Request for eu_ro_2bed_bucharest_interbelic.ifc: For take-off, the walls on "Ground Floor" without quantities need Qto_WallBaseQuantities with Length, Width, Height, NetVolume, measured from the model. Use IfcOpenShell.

First a look at what the model holds.

```python
import ifcopenshell
import ifcopenshell.util.element
import ifcopenshell.util.unit

model = ifcopenshell.open("eu_ro_2bed_bucharest_interbelic.ifc")
print(model.schema)
for unit_type in ("LENGTHUNIT", "AREAUNIT", "VOLUMEUNIT"):
    print(unit_type, ifcopenshell.util.unit.calculate_unit_scale(model, unit_type))
storey = next(s for s in model.by_type("IfcBuildingStorey") if s.Name == "Ground Floor")
walls = [e for e in ifcopenshell.util.element.get_decomposition(storey) if e.is_a("IfcWall")]
for e in sorted(walls, key=lambda e: e.id()):
    print(e.id(), e.is_a(), e.Name, list(ifcopenshell.util.element.get_psets(e, qtos_only=True)), sep=" | ")
```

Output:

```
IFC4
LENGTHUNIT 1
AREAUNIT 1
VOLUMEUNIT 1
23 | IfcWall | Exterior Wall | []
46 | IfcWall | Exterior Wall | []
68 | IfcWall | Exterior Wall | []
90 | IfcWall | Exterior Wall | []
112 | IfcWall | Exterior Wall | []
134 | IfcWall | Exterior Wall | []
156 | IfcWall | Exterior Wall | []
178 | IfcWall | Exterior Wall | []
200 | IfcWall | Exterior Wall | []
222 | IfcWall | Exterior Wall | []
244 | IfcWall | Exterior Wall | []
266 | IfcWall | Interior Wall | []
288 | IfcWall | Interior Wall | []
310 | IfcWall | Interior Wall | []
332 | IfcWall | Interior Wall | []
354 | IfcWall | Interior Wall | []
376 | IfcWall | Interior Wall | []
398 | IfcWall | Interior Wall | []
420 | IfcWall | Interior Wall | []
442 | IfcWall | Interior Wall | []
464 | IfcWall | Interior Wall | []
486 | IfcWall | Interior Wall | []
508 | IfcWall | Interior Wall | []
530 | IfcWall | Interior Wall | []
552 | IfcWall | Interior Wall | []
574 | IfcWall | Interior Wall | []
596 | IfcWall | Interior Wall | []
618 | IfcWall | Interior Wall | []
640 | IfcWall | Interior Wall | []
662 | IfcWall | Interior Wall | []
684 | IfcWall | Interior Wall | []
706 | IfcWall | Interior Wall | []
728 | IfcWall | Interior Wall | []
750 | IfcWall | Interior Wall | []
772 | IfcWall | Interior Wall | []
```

```python
import ifcopenshell
import ifcopenshell.api.pset
import ifcopenshell.geom
import ifcopenshell.util.element
import ifcopenshell.util.shape
import ifcopenshell.util.unit

model = ifcopenshell.open("eu_ro_2bed_bucharest_interbelic.ifc")
unit_scale = ifcopenshell.util.unit.calculate_unit_scale(model)
volume_scale = ifcopenshell.util.unit.calculate_unit_scale(model, "VOLUMEUNIT")
settings = ifcopenshell.geom.settings()

storey = next(s for s in model.by_type("IfcBuildingStorey") if s.Name == "Ground Floor")
walls = [e for e in ifcopenshell.util.element.get_decomposition(storey) if e.is_a("IfcWall")]

for e in sorted(walls, key=lambda e: e.id()):
    if ifcopenshell.util.element.get_psets(e, qtos_only=True, should_inherit=False):
        continue
    # Geometry comes back in metres, in the element's own axes.
    shape = ifcopenshell.geom.create_shape(settings, e)
    values = {
        "Length": ifcopenshell.util.shape.get_x(shape.geometry) / unit_scale,
        "Width": ifcopenshell.util.shape.get_y(shape.geometry) / unit_scale,
        "Height": ifcopenshell.util.shape.get_z(shape.geometry) / unit_scale,
        "NetVolume": ifcopenshell.util.shape.get_volume(shape.geometry) / volume_scale,
    }
    qto = ifcopenshell.api.pset.add_qto(model, product=e, name="Qto_WallBaseQuantities")
    ifcopenshell.api.pset.edit_qto(model, qto=qto, properties=values)
    print(e.id(), {k: round(v, 3) for k, v in values.items()})

model.write("eu_ro_2bed_bucharest_interbelic_updated.ifc")
```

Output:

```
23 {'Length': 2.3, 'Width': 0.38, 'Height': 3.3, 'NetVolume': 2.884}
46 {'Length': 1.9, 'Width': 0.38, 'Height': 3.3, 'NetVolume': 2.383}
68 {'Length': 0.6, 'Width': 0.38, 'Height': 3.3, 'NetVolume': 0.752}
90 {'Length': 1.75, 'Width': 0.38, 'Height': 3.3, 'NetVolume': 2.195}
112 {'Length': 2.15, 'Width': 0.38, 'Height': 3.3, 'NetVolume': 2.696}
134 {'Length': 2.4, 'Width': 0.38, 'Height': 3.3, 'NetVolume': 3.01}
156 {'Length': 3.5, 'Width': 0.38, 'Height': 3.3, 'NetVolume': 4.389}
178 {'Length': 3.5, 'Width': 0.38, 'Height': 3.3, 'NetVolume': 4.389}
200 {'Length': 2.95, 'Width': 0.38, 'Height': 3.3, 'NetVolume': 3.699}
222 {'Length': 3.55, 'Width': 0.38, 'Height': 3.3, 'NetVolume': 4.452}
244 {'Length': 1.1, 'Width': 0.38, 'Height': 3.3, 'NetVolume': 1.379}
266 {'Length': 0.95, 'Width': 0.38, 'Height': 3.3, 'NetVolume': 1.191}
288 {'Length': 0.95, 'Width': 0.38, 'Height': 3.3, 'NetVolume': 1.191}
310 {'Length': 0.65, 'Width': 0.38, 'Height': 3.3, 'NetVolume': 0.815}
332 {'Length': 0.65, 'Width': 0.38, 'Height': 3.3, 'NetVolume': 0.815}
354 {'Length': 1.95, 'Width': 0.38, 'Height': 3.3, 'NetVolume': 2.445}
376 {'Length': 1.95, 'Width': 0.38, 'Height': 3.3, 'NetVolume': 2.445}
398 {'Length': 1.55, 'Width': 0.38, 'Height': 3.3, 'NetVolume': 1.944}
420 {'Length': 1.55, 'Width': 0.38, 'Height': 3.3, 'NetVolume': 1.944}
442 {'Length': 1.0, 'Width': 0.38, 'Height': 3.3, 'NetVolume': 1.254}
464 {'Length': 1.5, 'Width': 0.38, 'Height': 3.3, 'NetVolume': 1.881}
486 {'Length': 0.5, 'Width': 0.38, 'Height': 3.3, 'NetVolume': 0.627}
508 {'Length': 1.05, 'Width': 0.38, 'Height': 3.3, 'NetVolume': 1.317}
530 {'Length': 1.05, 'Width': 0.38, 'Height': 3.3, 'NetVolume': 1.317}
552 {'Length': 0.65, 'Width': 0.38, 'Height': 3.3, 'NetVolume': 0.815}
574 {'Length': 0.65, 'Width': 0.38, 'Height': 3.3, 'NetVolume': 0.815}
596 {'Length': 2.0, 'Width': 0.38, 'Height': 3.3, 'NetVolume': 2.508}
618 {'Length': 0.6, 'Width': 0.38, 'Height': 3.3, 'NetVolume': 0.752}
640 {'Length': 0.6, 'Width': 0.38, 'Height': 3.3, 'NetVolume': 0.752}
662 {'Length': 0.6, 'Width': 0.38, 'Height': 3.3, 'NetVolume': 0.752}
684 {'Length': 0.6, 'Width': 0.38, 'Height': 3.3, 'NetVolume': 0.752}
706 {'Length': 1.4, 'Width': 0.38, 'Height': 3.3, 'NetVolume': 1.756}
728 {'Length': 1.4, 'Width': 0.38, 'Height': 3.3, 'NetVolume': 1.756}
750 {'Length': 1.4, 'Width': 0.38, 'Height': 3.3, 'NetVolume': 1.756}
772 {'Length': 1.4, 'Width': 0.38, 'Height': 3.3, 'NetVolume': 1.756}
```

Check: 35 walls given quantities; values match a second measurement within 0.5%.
